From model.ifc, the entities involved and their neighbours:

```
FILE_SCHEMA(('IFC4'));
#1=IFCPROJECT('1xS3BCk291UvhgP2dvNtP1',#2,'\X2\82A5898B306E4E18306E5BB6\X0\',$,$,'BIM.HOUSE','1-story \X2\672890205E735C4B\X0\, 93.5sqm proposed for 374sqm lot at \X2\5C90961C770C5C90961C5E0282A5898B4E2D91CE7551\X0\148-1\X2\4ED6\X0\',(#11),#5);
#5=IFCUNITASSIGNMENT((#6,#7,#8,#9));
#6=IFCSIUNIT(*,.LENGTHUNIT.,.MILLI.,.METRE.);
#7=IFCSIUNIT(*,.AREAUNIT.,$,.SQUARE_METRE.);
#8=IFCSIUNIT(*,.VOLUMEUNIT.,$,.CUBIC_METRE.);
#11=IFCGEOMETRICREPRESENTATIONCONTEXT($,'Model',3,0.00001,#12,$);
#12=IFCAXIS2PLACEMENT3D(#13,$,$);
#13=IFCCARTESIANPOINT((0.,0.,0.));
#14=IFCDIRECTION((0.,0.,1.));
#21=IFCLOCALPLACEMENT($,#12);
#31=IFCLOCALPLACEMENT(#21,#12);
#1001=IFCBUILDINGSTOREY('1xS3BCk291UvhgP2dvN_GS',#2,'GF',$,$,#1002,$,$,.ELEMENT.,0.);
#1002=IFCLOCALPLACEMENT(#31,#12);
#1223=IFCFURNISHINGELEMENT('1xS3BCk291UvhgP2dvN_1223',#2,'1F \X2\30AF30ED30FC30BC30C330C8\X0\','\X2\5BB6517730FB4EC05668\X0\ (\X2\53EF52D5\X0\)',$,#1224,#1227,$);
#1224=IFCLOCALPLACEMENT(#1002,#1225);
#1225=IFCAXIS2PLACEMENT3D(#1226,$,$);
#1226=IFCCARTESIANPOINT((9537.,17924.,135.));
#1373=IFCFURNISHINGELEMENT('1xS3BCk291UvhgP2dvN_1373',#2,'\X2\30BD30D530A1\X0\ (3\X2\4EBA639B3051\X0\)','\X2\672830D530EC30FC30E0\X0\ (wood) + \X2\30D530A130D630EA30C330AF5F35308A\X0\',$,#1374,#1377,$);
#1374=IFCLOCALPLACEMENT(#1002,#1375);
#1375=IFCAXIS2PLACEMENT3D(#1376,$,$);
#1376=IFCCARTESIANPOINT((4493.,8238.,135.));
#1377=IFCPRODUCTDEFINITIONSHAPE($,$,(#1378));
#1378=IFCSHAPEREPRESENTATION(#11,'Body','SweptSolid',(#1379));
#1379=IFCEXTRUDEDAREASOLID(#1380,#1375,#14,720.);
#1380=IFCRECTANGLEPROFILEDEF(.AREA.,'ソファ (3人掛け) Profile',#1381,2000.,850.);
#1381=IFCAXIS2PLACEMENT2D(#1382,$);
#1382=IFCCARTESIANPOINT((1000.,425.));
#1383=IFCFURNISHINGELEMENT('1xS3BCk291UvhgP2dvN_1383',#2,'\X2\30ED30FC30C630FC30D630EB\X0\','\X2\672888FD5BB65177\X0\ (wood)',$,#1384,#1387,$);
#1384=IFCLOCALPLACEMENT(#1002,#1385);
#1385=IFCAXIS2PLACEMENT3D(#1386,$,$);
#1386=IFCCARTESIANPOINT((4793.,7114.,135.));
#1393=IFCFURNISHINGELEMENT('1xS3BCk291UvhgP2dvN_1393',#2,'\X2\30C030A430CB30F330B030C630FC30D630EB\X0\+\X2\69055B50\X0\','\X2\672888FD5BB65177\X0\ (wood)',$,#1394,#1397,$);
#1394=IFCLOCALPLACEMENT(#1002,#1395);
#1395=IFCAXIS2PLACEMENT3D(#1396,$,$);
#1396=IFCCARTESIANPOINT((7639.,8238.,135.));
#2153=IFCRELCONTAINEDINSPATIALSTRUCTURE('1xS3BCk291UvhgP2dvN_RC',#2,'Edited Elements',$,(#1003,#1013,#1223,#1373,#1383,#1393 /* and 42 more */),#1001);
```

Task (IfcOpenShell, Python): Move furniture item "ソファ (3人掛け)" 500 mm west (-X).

```python
import ifcopenshell
import ifcopenshell.api.geometry
import ifcopenshell.util.placement
import ifcopenshell.util.unit

model = ifcopenshell.open("model.ifc")
unit_scale = ifcopenshell.util.unit.calculate_unit_scale(model)

item = model.by_guid("1xS3BCk291UvhgP2dvN_1373")
matrix = ifcopenshell.util.placement.get_local_placement(item.ObjectPlacement)
matrix[0, 3] -= 0.5 / unit_scale
ifcopenshell.api.geometry.edit_object_placement(model, product=item, matrix=matrix, is_si=False)

print(ifcopenshell.util.placement.get_local_placement(item.ObjectPlacement).round(3) + 0.0)

model.write("model_edited.ifc")
```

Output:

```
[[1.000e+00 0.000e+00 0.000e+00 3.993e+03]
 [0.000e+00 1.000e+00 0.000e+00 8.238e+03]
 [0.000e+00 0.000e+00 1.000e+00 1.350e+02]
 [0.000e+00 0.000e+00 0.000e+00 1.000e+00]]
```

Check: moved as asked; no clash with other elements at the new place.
